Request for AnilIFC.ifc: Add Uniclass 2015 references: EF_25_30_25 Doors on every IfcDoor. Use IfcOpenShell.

First a look at what the model holds.

```python
import ifcopenshell

model = ifcopenshell.open("AnilIFC.ifc")
print(model.schema)
print("classifications:", [c.Name for c in model.by_type("IfcClassification")])
for ifc_class in ("IfcDoor", "IfcRoof", "IfcStair", "IfcWall", "IfcWindow"):
    print(ifc_class, len(model.by_type(ifc_class)))
```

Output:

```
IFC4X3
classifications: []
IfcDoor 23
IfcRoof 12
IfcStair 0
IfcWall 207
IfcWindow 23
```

```python
import ifcopenshell
import ifcopenshell.api.classification

model = ifcopenshell.open("AnilIFC.ifc")

system = ifcopenshell.api.classification.add_classification(model, classification="Uniclass 2015")

codes = {
    "IfcDoor": ("EF_25_30_25", "Doors"),
}
for ifc_class, (code, name) in codes.items():
    products = model.by_type(ifc_class)
    ifcopenshell.api.classification.add_reference(
        model, products=products, classification=system, identification=code, name=name
    )
    print(code, len(products))

model.write("AnilIFC_updated.ifc")
```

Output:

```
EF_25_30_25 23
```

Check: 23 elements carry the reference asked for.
